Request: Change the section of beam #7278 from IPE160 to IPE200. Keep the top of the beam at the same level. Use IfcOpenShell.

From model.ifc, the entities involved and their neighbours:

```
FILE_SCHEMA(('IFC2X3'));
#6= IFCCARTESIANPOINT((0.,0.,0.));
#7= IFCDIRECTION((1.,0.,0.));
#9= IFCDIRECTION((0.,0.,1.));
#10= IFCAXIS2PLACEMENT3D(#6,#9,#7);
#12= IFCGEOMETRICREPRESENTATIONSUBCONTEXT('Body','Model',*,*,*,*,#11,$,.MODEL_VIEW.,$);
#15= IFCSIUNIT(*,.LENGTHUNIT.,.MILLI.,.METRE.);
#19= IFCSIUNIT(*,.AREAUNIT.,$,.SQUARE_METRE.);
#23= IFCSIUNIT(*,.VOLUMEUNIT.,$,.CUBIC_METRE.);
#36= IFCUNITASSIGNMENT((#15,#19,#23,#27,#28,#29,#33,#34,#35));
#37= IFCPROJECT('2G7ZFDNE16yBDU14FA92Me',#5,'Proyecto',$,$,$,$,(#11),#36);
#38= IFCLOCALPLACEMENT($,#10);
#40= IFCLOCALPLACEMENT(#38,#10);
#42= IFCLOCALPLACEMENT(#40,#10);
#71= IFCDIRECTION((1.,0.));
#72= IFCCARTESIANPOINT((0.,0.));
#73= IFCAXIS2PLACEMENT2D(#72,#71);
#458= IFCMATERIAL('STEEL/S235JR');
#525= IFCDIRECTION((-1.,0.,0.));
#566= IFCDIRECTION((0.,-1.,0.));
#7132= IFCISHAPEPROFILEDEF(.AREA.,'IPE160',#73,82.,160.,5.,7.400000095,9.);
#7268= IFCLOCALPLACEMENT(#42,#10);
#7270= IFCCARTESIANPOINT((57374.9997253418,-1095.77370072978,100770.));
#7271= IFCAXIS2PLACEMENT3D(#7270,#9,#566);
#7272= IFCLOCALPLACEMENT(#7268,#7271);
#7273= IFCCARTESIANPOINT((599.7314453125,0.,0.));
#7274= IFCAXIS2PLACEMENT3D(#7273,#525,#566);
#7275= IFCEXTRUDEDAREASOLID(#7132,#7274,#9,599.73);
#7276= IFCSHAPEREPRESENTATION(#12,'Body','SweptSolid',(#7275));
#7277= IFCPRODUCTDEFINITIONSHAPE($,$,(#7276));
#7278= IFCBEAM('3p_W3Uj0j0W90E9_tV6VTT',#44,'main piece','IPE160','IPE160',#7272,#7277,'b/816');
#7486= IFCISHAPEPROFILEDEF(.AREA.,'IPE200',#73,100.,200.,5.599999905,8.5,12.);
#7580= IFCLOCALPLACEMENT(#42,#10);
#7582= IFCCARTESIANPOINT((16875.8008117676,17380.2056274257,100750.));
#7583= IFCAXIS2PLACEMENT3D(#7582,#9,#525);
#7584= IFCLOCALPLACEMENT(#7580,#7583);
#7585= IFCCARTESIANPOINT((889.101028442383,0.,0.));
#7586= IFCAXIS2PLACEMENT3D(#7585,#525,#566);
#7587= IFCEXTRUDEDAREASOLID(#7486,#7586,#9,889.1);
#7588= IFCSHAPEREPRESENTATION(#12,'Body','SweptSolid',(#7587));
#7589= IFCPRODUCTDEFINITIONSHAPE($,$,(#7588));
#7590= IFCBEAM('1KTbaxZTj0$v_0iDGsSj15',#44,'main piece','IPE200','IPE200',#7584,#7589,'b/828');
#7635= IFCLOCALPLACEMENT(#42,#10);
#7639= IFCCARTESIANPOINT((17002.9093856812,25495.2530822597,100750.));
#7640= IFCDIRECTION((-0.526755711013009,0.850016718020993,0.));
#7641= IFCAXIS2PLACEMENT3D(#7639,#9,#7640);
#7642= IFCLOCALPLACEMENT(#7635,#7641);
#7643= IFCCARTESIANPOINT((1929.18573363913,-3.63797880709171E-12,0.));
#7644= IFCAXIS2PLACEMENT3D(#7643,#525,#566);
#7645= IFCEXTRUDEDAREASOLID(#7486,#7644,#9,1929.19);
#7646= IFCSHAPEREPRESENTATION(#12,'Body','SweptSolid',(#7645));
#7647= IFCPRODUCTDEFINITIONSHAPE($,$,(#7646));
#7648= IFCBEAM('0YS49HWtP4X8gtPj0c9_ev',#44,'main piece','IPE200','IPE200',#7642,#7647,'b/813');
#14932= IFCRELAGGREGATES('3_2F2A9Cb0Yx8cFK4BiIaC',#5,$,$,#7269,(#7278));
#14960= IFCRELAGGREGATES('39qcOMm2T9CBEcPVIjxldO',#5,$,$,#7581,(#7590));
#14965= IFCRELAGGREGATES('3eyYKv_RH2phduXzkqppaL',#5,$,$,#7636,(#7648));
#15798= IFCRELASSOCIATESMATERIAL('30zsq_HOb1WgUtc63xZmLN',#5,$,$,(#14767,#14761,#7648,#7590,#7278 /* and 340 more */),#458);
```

```python
import ifcopenshell
import ifcopenshell.util.element
import ifcopenshell.util.representation

model = ifcopenshell.open("model.ifc")

member = model.by_id(7278)
source = next(p for p in model.by_type("IfcIShapeProfileDef") if p.ProfileName == "IPE200")

body = ifcopenshell.util.representation.get_representation(member, "Model", "Body")
solid = body.Items[0]
old_profile = solid.SweptArea

# Copy the section's sizes but keep this member's own profile position.
profile = ifcopenshell.util.element.copy(model, source)
# Profiles are centred, so shift by half the change in depth to hold the top.
shift = (old_profile.OverallDepth - profile.OverallDepth) / 2
x, y = old_profile.Position.Location.Coordinates
up = (0.0, 1.0)  # upwards, in the solid's own plane
location = model.createIfcCartesianPoint((x + up[0] * shift, y + up[1] * shift))
profile.Position = model.createIfcAxis2Placement2D(location, old_profile.Position.RefDirection)
solid.SweptArea = profile
if not model.get_total_inverses(old_profile):
    ifcopenshell.util.element.remove_deep2(model, old_profile)
member.Description = member.Description.replace("IPE160", "IPE200")
member.ObjectType = member.ObjectType.replace("IPE160", "IPE200")

print(solid.SweptArea)

model.write("model-out.ifc")
```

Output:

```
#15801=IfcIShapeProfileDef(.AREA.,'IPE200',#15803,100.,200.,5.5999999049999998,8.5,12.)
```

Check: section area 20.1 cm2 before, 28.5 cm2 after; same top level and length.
